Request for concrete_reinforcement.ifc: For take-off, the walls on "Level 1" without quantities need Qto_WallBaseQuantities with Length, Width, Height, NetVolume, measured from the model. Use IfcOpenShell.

First a look at what the model holds.

```python
import ifcopenshell
import ifcopenshell.util.element
import ifcopenshell.util.unit

model = ifcopenshell.open("concrete_reinforcement.ifc")
print(model.schema)
for unit_type in ("LENGTHUNIT", "AREAUNIT", "VOLUMEUNIT"):
    print(unit_type, ifcopenshell.util.unit.calculate_unit_scale(model, unit_type))
storey = next(s for s in model.by_type("IfcBuildingStorey") if s.Name == "Level 1")
walls = [e for e in ifcopenshell.util.element.get_decomposition(storey) if e.is_a("IfcWall")]
for e in sorted(walls, key=lambda e: e.id()):
    print(e.id(), e.is_a(), e.Name, list(ifcopenshell.util.element.get_psets(e, qtos_only=True)), sep=" | ")
```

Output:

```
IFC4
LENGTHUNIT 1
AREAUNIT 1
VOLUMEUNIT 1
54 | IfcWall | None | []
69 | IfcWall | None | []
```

```python
import ifcopenshell
import ifcopenshell.api.pset
import ifcopenshell.geom
import ifcopenshell.util.element
import ifcopenshell.util.shape
import ifcopenshell.util.unit

model = ifcopenshell.open("concrete_reinforcement.ifc")
unit_scale = ifcopenshell.util.unit.calculate_unit_scale(model)
volume_scale = ifcopenshell.util.unit.calculate_unit_scale(model, "VOLUMEUNIT")
settings = ifcopenshell.geom.settings()

storey = next(s for s in model.by_type("IfcBuildingStorey") if s.Name == "Level 1")
walls = [e for e in ifcopenshell.util.element.get_decomposition(storey) if e.is_a("IfcWall")]

for e in sorted(walls, key=lambda e: e.id()):
    if ifcopenshell.util.element.get_psets(e, qtos_only=True, should_inherit=False):
        continue
    # Geometry comes back in metres, in the element's own axes.
    shape = ifcopenshell.geom.create_shape(settings, e)
    values = {
        "Length": ifcopenshell.util.shape.get_x(shape.geometry) / unit_scale,
        "Width": ifcopenshell.util.shape.get_y(shape.geometry) / unit_scale,
        "Height": ifcopenshell.util.shape.get_z(shape.geometry) / unit_scale,
        "NetVolume": ifcopenshell.util.shape.get_volume(shape.geometry) / volume_scale,
    }
    qto = ifcopenshell.api.pset.add_qto(model, product=e, name="Qto_WallBaseQuantities")
    ifcopenshell.api.pset.edit_qto(model, qto=qto, properties=values)
    print(e.id(), {k: round(v, 3) for k, v in values.items()})

model.write("concrete_reinforcement_v2.ifc")
```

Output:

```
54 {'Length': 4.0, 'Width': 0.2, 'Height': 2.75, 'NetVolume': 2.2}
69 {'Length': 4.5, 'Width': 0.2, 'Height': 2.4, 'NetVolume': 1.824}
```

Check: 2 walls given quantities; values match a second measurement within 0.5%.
